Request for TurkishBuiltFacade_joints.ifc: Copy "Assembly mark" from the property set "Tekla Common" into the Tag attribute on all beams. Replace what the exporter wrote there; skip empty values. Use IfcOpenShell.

First a look at what the model holds.

```python
import ifcopenshell
import ifcopenshell.util.element

model = ifcopenshell.open("TurkishBuiltFacade_joints.ifc")
print(model.schema)
beams = model.by_type("IfcBeam")
print(len(beams), "beams")
for e in beams[:8]:
    source = ifcopenshell.util.element.get_pset(e, "Tekla Common", "Assembly mark")
    target = e.Tag
    print(e.id(), repr(source), repr(target), sep=" | ")
```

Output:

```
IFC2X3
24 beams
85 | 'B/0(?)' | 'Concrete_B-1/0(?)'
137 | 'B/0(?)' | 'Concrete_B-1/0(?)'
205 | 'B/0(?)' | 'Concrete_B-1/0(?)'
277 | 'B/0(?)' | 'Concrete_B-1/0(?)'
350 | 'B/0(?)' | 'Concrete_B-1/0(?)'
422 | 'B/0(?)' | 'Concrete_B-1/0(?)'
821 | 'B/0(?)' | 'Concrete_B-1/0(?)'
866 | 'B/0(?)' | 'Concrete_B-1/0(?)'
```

```python
import ifcopenshell
import ifcopenshell.util.element

model = ifcopenshell.open("TurkishBuiltFacade_joints.ifc")

count = 0
for e in model.by_type("IfcBeam"):
    value = ifcopenshell.util.element.get_pset(e, "Tekla Common", "Assembly mark")
    current = e.Tag
    if not value or not value.strip() or current == value:
        continue
    e.Tag = value
    count += 1

print(count, "beams updated")

model.write("TurkishBuiltFacade_joints_v2.ifc")
```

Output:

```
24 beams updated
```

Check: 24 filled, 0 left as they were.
